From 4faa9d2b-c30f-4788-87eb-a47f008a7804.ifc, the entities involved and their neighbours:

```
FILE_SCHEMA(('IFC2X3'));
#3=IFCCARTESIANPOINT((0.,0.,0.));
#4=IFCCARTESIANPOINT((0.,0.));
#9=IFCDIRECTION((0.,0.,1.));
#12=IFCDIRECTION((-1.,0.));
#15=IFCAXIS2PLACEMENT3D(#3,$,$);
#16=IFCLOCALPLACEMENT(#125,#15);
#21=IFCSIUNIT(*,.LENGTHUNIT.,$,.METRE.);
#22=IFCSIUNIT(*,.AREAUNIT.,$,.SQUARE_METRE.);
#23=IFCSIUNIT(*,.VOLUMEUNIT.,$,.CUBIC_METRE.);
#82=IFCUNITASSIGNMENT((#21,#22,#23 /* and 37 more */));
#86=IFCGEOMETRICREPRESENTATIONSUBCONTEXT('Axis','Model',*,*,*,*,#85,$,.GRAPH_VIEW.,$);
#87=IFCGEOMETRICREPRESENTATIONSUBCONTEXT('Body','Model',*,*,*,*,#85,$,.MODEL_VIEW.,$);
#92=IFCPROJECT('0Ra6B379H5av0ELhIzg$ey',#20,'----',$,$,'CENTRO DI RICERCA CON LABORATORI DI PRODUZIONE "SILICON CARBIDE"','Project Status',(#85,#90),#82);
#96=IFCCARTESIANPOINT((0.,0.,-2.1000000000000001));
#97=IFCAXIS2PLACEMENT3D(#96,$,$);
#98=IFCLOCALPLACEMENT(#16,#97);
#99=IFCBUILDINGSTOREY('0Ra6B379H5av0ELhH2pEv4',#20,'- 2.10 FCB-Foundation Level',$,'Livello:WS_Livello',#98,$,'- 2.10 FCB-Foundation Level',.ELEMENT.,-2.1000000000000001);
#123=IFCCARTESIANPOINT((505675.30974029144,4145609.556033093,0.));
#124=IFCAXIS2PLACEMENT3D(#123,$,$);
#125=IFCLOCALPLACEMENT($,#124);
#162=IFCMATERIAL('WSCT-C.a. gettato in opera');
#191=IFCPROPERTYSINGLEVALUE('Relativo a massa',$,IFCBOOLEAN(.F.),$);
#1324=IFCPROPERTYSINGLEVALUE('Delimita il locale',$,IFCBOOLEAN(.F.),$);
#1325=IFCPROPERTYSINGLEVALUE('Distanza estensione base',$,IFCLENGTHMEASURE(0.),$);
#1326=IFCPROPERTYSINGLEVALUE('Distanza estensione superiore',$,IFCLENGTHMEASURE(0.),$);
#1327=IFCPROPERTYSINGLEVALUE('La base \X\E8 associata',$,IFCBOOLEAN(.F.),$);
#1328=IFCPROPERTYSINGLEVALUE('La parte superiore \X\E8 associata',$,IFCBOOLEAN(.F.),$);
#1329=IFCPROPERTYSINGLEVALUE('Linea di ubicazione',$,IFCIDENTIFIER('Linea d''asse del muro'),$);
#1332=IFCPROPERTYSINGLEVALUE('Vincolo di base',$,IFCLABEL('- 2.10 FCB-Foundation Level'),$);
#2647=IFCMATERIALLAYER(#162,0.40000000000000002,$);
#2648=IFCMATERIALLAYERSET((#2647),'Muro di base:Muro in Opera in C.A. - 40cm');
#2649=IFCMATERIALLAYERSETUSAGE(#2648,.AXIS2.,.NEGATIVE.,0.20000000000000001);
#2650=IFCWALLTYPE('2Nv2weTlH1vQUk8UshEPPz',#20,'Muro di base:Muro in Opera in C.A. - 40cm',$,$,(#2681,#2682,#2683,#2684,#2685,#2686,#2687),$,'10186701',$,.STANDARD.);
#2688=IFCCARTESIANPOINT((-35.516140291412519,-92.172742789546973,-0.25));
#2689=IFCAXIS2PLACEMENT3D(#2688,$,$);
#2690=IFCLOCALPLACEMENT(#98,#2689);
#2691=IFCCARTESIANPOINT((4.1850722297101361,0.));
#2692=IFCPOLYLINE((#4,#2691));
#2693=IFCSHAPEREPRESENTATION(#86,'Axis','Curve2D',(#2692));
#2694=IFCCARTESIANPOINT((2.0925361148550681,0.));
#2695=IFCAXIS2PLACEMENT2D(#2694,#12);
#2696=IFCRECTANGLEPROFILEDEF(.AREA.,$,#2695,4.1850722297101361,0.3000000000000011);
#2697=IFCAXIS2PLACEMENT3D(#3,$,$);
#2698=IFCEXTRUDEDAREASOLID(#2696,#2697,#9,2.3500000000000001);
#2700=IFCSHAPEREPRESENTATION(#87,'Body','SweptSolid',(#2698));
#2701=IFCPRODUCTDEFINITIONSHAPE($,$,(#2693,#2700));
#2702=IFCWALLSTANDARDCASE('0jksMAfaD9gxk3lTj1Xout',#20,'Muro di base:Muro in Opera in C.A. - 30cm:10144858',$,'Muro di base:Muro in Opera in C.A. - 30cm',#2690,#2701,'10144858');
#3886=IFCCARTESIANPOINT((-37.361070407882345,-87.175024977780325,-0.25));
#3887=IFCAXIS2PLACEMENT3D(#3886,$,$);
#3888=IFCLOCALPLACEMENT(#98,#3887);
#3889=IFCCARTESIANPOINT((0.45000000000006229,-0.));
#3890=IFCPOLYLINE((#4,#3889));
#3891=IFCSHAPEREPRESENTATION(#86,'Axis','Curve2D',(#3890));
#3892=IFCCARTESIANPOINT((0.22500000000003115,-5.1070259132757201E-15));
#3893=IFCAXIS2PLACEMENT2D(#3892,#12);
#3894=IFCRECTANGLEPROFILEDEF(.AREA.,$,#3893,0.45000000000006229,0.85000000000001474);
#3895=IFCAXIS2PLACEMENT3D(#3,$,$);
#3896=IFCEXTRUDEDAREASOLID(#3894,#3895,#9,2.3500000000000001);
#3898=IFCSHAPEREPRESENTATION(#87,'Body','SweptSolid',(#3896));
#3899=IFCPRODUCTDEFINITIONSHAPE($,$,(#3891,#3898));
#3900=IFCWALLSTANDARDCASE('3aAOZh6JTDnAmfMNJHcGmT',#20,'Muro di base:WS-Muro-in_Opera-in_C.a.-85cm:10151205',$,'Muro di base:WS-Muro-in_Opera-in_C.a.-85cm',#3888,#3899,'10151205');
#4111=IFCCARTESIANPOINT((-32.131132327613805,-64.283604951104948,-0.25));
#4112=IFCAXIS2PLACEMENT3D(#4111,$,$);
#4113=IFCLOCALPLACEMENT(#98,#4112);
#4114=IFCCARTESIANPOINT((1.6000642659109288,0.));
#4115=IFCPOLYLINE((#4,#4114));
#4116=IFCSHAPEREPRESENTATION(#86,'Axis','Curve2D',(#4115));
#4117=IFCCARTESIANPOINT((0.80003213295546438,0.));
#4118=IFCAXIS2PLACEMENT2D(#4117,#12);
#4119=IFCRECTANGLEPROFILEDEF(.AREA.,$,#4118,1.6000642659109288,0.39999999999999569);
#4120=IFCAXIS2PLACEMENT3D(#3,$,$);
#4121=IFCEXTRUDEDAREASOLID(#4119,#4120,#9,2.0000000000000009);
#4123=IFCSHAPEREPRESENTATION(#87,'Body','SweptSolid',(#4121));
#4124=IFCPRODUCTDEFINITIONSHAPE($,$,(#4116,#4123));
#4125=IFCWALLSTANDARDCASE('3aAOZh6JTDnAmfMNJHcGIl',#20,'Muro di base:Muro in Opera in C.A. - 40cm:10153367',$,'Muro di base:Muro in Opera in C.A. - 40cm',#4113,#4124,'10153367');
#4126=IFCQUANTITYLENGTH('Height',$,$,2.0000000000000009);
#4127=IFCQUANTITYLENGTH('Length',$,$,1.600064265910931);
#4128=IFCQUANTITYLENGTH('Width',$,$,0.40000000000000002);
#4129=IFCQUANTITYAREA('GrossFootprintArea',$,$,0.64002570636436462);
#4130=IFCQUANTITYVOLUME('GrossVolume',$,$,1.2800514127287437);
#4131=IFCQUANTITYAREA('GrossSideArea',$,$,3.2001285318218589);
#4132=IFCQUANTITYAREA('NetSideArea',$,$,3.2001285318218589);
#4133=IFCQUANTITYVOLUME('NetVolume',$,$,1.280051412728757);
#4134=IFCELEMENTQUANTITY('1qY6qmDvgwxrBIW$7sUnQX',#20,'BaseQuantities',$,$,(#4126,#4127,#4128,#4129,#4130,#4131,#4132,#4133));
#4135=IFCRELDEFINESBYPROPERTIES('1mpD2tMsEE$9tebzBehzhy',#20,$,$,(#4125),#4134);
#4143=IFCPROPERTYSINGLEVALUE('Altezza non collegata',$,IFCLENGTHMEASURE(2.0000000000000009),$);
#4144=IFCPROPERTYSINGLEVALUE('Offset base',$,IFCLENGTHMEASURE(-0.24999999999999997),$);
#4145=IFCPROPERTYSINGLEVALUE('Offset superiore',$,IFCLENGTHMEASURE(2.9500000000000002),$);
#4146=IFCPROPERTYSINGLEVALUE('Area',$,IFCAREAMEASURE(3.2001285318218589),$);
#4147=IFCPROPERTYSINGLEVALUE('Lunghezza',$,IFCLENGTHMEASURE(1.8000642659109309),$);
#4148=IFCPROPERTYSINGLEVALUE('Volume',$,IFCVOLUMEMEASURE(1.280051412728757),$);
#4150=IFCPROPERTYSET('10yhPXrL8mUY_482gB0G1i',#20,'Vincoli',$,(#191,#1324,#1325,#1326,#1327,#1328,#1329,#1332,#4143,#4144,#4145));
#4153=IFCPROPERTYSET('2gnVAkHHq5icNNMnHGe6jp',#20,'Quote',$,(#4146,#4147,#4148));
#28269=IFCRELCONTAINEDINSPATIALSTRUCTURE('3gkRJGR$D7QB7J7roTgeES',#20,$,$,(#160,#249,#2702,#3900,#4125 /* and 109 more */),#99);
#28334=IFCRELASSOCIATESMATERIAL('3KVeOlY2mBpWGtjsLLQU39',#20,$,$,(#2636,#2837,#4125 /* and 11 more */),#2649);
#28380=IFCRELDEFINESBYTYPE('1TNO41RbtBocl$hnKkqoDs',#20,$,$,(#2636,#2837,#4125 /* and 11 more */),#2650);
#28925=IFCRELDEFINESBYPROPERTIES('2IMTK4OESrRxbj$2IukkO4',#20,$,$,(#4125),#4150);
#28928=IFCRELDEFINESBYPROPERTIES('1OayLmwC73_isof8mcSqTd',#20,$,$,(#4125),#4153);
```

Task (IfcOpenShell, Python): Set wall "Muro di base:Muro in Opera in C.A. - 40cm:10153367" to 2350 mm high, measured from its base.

```python
import ifcopenshell
import ifcopenshell.api.pset
import ifcopenshell.geom
import ifcopenshell.util.element
import ifcopenshell.util.representation
import ifcopenshell.util.shape
import ifcopenshell.util.unit

model = ifcopenshell.open("4faa9d2b-c30f-4788-87eb-a47f008a7804.ifc")
unit_scale = ifcopenshell.util.unit.calculate_unit_scale(model)
area_scale = ifcopenshell.util.unit.calculate_unit_scale(model, "AREAUNIT")
volume_scale = ifcopenshell.util.unit.calculate_unit_scale(model, "VOLUMEUNIT")
settings = ifcopenshell.geom.settings()


def volume(element):
    """Net volume in cubic metres, openings subtracted."""
    shape = ifcopenshell.geom.create_shape(settings, element)
    return ifcopenshell.util.shape.get_volume(shape.geometry)


wall = model.by_guid("3aAOZh6JTDnAmfMNJHcGIl")
before = volume(wall)

body = ifcopenshell.util.representation.get_representation(wall, "Model", "Body")
solid = body.Items[0]
old_height = solid.Depth
solid.Depth = 2.35 / unit_scale
after = volume(wall)
thickness = 0.4  # wall thickness in metres

# Update the stored height, areas and volumes.
qto = model.by_id(ifcopenshell.util.element.get_pset(wall, "BaseQuantities", should_inherit=False)["id"])
ifcopenshell.api.pset.edit_qto(model, qto=qto, properties={
    "Height": solid.Depth,
    "GrossVolume": ifcopenshell.util.element.get_pset(wall, "BaseQuantities", "GrossVolume") * solid.Depth / old_height,
    "GrossSideArea": ifcopenshell.util.element.get_pset(wall, "BaseQuantities", "GrossSideArea") * solid.Depth / old_height,
    "NetSideArea": after / thickness / area_scale,
    "NetVolume": after / volume_scale,
})
pset = model.by_id(ifcopenshell.util.element.get_pset(wall, "Vincoli", should_inherit=False)["id"])
ifcopenshell.api.pset.edit_pset(model, pset=pset, properties={
    "Altezza non collegata": model.create_entity("IfcLengthMeasure", solid.Depth),
})
pset = model.by_id(ifcopenshell.util.element.get_pset(wall, "Quote", should_inherit=False)["id"])
ifcopenshell.api.pset.edit_pset(model, pset=pset, properties={
    "Area": model.create_entity("IfcAreaMeasure", after / thickness / area_scale),
    "Volume": model.create_entity("IfcVolumeMeasure", after / volume_scale),
})

print(f"height {old_height:g} -> {solid.Depth:g}, volume {before:.3f} -> {after:.3f} m3")

model.write("4faa9d2b-c30f-4788-87eb-a47f008a7804-out.ifc")
```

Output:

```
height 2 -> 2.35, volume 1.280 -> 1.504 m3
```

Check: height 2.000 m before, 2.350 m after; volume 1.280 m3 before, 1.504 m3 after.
